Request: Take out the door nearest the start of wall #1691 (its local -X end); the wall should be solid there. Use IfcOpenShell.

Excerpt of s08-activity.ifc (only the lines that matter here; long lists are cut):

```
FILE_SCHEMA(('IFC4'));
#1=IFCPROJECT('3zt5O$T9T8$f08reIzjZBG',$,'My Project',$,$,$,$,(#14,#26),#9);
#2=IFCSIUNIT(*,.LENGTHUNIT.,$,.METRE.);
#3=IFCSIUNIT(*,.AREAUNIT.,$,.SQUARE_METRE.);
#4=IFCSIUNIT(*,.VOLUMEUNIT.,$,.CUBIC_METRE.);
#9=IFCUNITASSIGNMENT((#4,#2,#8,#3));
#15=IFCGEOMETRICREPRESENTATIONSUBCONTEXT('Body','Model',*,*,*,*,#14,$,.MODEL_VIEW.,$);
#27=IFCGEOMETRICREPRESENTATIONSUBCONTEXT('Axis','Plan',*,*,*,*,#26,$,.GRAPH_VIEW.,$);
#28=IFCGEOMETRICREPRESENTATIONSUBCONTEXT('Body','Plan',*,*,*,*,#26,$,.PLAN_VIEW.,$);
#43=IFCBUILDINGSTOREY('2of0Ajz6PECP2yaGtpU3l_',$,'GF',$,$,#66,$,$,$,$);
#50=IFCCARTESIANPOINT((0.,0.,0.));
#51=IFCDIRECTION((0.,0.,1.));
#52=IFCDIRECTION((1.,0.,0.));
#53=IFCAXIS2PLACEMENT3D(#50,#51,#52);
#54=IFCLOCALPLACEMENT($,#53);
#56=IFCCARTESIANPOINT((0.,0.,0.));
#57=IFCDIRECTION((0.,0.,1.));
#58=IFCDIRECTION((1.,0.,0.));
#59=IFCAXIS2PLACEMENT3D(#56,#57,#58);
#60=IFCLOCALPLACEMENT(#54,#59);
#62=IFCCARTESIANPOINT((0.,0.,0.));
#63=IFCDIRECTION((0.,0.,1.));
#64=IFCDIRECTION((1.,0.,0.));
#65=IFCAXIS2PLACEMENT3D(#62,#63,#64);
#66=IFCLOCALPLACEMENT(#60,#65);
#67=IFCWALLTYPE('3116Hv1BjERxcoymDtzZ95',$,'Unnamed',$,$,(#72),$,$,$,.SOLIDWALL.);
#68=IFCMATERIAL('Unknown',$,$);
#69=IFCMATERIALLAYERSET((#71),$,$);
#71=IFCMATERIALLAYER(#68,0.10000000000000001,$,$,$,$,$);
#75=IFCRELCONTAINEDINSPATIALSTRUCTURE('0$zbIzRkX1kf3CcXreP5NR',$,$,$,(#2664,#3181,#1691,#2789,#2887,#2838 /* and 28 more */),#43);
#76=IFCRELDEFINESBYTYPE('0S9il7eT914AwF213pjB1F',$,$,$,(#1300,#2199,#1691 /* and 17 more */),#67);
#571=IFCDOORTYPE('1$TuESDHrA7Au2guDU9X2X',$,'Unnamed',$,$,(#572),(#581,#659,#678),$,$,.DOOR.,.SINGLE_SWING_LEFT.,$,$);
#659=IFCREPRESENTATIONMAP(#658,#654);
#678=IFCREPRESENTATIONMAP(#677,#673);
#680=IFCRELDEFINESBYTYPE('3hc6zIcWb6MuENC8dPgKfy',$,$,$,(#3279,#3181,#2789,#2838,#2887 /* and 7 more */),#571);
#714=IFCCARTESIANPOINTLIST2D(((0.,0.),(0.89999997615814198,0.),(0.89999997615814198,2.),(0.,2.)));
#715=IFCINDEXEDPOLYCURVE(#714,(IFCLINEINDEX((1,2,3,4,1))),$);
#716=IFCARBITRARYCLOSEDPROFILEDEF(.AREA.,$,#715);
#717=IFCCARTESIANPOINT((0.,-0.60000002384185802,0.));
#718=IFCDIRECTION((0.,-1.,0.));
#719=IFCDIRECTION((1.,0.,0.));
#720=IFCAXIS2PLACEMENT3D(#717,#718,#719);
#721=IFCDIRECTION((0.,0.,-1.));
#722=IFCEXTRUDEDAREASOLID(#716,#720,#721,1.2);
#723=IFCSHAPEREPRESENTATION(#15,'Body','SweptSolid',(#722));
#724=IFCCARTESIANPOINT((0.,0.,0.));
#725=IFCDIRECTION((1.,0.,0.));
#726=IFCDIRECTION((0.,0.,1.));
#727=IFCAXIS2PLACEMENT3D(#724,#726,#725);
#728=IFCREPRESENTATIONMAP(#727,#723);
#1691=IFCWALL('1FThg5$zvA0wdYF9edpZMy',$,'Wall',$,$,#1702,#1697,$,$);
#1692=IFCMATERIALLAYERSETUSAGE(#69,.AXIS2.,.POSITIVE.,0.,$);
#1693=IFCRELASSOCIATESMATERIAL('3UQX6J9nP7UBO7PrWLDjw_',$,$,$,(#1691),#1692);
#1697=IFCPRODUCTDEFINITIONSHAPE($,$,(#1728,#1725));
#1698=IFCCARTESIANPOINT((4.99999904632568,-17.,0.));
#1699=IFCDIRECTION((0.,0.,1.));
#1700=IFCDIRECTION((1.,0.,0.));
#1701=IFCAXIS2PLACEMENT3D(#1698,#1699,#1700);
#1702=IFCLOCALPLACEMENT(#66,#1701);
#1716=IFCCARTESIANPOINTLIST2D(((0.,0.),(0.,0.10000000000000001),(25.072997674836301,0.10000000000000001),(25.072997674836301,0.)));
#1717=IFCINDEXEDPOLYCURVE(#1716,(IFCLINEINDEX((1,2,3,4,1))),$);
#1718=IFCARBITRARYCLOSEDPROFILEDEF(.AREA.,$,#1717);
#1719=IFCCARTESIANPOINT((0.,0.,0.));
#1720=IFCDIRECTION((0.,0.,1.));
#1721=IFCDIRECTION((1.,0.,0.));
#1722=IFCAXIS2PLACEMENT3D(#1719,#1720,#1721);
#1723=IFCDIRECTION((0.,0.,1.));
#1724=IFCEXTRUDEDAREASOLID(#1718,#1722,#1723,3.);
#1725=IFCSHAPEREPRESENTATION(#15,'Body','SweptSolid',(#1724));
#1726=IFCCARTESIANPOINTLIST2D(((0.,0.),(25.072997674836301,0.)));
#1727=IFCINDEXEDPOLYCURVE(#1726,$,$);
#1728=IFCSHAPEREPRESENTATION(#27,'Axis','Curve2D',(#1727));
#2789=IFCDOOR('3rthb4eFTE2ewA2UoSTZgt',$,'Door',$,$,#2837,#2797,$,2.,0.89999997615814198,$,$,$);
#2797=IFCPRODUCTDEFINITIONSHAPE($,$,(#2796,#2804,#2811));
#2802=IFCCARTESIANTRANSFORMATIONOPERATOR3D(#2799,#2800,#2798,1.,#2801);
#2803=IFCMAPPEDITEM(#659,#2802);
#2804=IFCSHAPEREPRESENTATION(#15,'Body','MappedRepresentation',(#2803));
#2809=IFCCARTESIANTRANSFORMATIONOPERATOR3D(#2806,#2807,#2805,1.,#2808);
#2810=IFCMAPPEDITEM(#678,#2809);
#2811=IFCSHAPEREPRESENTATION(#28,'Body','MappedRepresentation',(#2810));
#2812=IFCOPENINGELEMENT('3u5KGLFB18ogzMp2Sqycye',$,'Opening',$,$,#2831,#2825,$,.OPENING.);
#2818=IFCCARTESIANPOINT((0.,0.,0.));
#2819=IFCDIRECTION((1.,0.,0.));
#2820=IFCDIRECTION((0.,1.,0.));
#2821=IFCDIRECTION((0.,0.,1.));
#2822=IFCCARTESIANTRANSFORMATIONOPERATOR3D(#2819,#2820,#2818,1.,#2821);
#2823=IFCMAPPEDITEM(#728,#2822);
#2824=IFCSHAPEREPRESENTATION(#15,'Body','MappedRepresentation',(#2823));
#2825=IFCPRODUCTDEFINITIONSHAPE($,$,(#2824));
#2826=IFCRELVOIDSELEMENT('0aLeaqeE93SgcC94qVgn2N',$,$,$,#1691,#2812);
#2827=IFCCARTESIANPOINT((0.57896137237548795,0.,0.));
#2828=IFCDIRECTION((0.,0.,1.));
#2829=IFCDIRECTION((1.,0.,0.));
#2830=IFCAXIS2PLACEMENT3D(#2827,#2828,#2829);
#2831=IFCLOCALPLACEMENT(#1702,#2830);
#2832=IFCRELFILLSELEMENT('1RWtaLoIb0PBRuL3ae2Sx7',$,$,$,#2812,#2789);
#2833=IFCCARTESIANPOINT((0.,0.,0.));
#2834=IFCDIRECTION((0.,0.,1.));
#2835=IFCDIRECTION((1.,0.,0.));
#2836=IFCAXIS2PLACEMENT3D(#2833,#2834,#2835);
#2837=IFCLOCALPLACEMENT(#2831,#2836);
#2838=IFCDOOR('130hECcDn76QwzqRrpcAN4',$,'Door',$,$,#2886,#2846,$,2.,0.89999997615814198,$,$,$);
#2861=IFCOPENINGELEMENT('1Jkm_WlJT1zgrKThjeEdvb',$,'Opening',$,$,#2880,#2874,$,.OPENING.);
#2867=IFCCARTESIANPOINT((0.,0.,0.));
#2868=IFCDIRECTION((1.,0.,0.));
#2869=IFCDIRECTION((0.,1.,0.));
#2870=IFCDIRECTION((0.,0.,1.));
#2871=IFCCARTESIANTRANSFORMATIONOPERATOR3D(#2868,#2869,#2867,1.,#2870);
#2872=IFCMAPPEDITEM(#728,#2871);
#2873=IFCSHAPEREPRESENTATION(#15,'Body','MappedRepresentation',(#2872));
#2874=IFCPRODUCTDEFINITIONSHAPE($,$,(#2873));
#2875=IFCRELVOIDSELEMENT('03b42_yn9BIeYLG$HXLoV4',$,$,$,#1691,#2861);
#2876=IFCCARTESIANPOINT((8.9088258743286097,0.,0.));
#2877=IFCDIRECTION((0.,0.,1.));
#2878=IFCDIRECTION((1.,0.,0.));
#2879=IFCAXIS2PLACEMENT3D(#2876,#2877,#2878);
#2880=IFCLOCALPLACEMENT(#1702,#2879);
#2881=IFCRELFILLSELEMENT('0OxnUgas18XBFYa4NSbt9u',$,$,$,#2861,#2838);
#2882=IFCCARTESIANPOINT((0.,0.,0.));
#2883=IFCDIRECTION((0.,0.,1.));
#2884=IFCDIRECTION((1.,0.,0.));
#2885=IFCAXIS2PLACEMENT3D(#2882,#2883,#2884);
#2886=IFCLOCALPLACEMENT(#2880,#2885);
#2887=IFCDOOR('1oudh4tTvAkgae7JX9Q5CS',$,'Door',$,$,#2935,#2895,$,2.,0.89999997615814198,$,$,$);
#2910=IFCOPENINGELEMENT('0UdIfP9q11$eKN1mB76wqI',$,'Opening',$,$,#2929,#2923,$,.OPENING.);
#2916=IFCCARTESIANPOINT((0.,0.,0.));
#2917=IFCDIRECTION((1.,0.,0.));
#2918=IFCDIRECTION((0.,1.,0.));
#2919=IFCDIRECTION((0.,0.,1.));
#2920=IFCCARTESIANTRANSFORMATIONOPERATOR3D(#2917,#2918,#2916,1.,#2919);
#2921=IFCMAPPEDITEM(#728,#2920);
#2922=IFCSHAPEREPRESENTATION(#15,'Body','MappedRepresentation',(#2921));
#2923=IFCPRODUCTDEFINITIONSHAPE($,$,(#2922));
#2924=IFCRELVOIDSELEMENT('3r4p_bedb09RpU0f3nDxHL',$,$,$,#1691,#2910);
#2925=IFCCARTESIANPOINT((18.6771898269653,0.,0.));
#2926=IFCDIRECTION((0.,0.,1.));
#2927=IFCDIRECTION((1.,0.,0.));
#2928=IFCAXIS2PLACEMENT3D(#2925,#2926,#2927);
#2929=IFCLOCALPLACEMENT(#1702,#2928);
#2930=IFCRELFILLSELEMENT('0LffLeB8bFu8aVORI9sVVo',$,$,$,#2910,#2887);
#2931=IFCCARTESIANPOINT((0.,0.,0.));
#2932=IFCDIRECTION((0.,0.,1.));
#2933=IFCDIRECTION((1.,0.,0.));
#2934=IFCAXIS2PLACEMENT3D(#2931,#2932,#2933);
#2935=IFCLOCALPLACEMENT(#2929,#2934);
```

```python
import ifcopenshell
import ifcopenshell.api.feature
import ifcopenshell.api.root
import ifcopenshell.geom
import ifcopenshell.util.shape

model = ifcopenshell.open("s08-activity.ifc")
settings = ifcopenshell.geom.settings()


def volume(element):
    """Net volume in cubic metres, openings subtracted."""
    shape = ifcopenshell.geom.create_shape(settings, element)
    return ifcopenshell.util.shape.get_volume(shape.geometry)


door = model.by_guid("3rthb4eFTE2ewA2UoSTZgt")
opening = door.FillsVoids[0].RelatingOpeningElement
wall = opening.VoidsElements[0].RelatingBuildingElement
before = volume(wall)

ifcopenshell.api.root.remove_product(model, product=door)
ifcopenshell.api.feature.remove_feature(model, feature=opening)

after = volume(wall)

print(f"wall volume {before:.3f} -> {after:.3f} m3")

model.write("s08-activity-out.ifc")
```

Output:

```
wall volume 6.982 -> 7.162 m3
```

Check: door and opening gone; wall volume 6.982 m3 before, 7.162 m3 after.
